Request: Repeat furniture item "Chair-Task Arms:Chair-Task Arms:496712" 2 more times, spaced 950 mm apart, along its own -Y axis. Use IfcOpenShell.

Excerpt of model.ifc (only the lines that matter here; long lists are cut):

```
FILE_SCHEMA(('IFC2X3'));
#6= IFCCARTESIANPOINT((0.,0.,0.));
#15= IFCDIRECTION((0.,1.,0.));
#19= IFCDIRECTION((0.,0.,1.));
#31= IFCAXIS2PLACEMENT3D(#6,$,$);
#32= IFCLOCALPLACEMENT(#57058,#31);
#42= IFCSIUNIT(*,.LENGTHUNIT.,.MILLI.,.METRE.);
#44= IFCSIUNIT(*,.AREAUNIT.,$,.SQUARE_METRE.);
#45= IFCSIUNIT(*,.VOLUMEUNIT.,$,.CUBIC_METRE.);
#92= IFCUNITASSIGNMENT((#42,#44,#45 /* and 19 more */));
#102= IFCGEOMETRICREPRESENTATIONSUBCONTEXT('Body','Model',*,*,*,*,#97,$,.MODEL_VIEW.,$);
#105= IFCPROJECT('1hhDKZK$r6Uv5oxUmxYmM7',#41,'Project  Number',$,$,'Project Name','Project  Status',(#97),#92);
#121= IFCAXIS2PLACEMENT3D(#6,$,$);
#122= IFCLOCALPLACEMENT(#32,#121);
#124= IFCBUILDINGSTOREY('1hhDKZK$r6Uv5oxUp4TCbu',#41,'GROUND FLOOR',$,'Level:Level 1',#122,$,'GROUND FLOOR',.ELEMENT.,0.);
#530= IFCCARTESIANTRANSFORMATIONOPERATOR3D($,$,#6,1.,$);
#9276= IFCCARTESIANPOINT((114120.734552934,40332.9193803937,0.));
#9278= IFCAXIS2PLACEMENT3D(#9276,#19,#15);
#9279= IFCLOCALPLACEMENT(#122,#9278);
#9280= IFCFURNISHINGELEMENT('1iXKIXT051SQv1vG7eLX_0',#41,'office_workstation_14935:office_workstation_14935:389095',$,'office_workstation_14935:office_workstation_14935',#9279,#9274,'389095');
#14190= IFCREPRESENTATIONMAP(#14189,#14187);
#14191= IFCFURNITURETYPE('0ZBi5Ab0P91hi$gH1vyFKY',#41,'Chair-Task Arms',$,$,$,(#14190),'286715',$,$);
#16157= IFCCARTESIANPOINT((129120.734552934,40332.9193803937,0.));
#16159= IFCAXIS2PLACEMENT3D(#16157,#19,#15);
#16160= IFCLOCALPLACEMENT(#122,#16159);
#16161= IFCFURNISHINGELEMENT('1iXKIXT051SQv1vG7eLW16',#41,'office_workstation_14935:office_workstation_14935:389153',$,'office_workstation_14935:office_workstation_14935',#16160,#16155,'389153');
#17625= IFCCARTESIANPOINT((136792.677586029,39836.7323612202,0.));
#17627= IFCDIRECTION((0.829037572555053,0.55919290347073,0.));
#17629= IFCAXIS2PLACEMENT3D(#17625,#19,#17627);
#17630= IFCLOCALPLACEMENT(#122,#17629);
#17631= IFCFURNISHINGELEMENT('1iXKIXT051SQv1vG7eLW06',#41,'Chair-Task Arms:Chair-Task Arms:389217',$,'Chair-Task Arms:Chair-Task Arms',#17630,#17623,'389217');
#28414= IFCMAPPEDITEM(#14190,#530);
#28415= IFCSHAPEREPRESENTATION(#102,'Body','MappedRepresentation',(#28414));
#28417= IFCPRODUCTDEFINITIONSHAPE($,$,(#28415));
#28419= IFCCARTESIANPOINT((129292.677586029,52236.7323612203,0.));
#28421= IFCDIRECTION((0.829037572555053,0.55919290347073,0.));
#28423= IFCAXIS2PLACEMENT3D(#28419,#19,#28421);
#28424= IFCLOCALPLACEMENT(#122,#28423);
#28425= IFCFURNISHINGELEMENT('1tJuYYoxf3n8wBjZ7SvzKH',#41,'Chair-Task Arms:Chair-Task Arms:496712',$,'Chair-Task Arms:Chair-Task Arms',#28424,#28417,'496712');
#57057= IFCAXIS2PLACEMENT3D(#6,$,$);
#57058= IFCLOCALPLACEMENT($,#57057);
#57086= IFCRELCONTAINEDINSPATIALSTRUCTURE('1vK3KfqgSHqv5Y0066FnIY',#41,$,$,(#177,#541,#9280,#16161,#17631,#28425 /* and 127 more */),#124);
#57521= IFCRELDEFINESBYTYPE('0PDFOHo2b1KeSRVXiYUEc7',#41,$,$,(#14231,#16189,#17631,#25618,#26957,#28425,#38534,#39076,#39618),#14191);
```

```python
import ifcopenshell
import ifcopenshell.api.geometry
import ifcopenshell.api.root
import ifcopenshell.util.element
import ifcopenshell.util.placement

model = ifcopenshell.open("model.ifc")


def reuse_history(source, copy):
    """copy_class also copies each property set's owner history, people and application; keep the originals."""
    for rel in copy.IsDefinedBy:
        if rel.is_a("IfcRelDefinesByProperties") and (history := rel.RelatingPropertyDefinition.OwnerHistory):
            rel.RelatingPropertyDefinition.OwnerHistory = source.OwnerHistory
            ifcopenshell.util.element.remove_deep2(model, history)


source = model.by_guid("1tJuYYoxf3n8wBjZ7SvzKH")
base = ifcopenshell.util.placement.get_local_placement(source.ObjectPlacement)
step = -base[:3, 1] * 950.0

for i in range(1, 3):
    copy = ifcopenshell.api.root.copy_class(model, product=source)
    copy.Representation = ifcopenshell.util.element.copy_deep(
        model, source.Representation, exclude=["IfcGeometricRepresentationContext", "IfcRepresentationMap"]
    )
    copy.Name = "Chair-Task Arms:Chair-Task Arms"
    copy.Tag = None
    reuse_history(source, copy)
    matrix = base.copy()
    matrix[:3, 3] += i * step
    print("added at", matrix[:3, 3].round(3) + 0.0)
    ifcopenshell.api.geometry.edit_object_placement(model, product=copy, matrix=matrix, is_si=False)

model.write("model_updated.ifc")
```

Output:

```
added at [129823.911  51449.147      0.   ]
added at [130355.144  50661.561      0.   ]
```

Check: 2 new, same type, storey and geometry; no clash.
